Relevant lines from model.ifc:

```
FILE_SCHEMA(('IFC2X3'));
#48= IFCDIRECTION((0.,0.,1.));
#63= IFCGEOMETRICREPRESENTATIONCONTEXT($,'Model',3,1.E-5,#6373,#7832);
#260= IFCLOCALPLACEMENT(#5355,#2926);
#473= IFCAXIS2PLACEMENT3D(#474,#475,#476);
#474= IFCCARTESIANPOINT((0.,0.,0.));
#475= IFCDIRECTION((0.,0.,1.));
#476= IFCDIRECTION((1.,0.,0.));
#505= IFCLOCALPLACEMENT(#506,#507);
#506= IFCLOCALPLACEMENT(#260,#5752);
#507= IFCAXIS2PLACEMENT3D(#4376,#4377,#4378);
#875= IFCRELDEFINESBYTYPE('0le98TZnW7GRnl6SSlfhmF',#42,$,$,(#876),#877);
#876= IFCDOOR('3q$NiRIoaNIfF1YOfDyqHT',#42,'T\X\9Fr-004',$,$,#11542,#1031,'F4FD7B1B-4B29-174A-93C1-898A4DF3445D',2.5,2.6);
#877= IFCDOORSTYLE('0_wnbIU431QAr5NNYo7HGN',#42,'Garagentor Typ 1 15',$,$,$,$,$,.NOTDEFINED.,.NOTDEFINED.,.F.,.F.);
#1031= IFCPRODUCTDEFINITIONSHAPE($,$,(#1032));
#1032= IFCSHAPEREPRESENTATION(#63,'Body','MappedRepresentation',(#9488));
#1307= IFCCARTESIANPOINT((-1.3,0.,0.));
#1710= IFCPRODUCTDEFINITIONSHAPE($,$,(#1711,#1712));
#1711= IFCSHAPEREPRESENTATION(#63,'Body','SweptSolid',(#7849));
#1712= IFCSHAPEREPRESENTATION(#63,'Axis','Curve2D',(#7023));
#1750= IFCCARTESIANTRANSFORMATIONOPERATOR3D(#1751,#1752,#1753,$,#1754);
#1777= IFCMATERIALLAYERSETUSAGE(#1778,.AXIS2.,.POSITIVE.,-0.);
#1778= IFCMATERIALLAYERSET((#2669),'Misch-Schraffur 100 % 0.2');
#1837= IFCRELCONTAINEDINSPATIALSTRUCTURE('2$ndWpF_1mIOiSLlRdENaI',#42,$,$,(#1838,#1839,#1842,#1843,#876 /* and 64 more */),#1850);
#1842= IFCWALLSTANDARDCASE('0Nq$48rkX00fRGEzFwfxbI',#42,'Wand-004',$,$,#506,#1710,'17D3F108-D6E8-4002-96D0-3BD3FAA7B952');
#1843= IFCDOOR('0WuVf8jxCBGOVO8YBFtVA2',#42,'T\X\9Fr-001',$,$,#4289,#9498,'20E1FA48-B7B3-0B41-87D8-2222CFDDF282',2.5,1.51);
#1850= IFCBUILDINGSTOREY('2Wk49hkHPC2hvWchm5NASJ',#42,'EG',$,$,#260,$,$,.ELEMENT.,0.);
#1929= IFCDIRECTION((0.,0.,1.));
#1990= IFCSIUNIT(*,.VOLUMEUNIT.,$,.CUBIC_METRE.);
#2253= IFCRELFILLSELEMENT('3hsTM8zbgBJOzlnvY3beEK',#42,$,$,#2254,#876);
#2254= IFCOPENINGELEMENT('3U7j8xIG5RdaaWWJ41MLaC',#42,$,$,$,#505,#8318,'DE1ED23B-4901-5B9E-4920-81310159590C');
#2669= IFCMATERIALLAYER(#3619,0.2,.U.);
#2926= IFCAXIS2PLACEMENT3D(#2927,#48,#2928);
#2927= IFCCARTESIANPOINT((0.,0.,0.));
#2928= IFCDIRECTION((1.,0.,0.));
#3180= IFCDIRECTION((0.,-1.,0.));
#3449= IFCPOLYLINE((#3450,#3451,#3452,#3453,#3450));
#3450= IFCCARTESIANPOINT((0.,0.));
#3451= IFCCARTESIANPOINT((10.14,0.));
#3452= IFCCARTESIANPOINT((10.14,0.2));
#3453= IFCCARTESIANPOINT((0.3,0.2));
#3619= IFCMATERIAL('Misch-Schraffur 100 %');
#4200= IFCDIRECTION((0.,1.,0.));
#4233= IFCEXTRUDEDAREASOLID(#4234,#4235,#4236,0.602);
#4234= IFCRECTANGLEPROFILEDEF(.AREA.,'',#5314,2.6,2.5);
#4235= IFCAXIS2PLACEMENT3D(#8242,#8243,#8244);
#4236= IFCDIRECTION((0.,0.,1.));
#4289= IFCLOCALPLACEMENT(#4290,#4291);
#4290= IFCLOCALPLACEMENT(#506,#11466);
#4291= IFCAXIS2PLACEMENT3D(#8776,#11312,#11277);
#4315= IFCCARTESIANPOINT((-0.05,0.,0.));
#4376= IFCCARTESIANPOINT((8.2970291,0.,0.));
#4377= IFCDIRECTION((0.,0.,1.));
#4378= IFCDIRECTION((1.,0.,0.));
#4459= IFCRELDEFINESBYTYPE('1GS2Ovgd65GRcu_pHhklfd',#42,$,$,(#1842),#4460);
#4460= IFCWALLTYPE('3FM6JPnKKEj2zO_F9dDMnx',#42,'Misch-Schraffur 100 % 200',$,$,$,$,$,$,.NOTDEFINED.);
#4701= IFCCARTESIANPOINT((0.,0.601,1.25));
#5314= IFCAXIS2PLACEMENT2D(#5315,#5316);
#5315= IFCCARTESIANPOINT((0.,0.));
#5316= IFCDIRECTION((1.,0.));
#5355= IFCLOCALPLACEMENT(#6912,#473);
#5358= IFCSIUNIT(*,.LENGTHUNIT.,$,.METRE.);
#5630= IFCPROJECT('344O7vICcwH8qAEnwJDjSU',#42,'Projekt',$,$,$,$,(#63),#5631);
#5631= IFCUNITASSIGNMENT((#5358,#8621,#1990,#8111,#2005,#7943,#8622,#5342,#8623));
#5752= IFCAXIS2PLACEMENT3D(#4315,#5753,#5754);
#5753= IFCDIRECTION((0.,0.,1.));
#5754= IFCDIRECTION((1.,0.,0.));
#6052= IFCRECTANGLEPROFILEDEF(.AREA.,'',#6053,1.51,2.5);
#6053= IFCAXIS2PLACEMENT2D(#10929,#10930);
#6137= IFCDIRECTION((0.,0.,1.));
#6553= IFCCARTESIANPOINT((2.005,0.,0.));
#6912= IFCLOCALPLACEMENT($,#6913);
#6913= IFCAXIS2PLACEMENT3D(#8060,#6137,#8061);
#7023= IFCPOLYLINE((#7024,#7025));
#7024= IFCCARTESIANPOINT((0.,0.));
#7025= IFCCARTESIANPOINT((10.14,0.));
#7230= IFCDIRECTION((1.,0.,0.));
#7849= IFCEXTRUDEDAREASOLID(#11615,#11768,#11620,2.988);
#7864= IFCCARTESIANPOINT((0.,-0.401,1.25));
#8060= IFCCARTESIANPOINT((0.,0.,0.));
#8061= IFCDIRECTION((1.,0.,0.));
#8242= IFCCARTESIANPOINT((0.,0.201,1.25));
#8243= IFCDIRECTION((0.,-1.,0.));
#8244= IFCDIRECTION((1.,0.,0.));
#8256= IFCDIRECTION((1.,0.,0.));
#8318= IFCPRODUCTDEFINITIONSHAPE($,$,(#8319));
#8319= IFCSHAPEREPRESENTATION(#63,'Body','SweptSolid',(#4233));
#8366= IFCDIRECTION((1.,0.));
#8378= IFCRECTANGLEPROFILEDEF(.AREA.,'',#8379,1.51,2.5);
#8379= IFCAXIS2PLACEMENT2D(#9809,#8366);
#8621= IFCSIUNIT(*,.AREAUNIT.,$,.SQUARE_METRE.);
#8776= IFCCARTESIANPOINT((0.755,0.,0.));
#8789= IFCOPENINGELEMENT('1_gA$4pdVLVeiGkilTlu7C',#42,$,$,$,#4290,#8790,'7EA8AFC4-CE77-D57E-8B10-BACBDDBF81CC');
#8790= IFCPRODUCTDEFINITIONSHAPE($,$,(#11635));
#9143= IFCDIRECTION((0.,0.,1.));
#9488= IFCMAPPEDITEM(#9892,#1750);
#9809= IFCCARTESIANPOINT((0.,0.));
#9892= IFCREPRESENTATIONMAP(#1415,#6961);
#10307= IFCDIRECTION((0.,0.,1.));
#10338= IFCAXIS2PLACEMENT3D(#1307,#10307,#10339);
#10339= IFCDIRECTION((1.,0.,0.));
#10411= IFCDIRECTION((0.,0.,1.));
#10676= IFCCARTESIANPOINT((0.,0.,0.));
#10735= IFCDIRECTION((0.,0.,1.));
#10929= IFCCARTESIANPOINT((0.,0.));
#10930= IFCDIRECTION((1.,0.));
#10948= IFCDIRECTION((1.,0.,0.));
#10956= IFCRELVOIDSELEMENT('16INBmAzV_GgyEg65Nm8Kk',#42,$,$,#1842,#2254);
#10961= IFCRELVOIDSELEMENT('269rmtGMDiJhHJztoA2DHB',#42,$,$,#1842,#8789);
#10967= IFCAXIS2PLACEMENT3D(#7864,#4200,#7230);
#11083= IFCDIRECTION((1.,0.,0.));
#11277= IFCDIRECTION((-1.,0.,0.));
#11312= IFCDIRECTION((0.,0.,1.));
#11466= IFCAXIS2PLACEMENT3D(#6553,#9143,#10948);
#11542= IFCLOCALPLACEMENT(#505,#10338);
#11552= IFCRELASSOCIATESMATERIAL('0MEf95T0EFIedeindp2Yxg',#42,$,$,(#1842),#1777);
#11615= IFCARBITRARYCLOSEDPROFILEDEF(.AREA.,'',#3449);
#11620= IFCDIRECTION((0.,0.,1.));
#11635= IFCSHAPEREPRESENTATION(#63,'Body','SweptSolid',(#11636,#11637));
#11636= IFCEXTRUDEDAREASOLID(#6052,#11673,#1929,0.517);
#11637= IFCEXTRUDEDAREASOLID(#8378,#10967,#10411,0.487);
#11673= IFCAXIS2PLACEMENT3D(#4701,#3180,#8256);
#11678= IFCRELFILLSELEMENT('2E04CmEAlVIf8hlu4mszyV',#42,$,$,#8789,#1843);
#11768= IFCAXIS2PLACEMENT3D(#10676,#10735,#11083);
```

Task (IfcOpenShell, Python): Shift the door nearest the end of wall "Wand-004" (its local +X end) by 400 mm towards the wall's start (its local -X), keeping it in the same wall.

```python
import ifcopenshell
import ifcopenshell.api.geometry
import ifcopenshell.util.placement
import ifcopenshell.util.unit

model = ifcopenshell.open("model.ifc")
unit_scale = ifcopenshell.util.unit.calculate_unit_scale(model)

door = model.by_guid("3q$NiRIoaNIfF1YOfDyqHT")
opening = door.FillsVoids[0].RelatingOpeningElement
wall = opening.VoidsElements[0].RelatingBuildingElement

wall_matrix = ifcopenshell.util.placement.get_local_placement(wall.ObjectPlacement)
shift = wall_matrix[:3, 0] * -0.4 / unit_scale
before = ifcopenshell.util.placement.get_local_placement(door.ObjectPlacement)[:3, 3].copy()

# The door is placed relative to its opening, so it follows when the opening moves.
matrix = ifcopenshell.util.placement.get_local_placement(opening.ObjectPlacement)
matrix[:3, 3] += shift
ifcopenshell.api.geometry.edit_object_placement(
    model, product=opening, matrix=matrix, is_si=False, should_transform_children=True
)

after = ifcopenshell.util.placement.get_local_placement(door.ObjectPlacement)[:3, 3]
print("door moved by", (after - before).round(3) + 0.0)

model.write("model_updated.ifc")
```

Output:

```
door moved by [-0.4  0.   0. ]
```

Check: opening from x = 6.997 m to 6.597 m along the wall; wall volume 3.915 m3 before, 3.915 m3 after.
